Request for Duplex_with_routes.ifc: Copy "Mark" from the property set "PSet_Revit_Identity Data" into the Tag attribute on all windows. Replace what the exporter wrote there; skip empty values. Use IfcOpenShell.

First a look at what the model holds.

```python
import ifcopenshell
import ifcopenshell.util.element

model = ifcopenshell.open("Duplex_with_routes.ifc")
print(model.schema)
windows = model.by_type("IfcWindow")
print(len(windows), "windows")
for e in windows[:8]:
    source = ifcopenshell.util.element.get_pset(e, "PSet_Revit_Identity Data", "Mark")
    target = e.Tag
    print(e.id(), repr(source), repr(target), sep=" | ")
```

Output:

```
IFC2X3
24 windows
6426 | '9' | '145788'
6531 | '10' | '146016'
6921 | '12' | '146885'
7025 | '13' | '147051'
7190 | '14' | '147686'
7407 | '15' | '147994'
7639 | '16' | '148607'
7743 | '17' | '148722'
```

```python
import ifcopenshell
import ifcopenshell.util.element

model = ifcopenshell.open("Duplex_with_routes.ifc")

count = 0
for e in model.by_type("IfcWindow"):
    value = ifcopenshell.util.element.get_pset(e, "PSet_Revit_Identity Data", "Mark")
    current = e.Tag
    if not value or not value.strip() or current == value:
        continue
    e.Tag = value
    count += 1

print(count, "windows updated")

model.write("Duplex_with_routes-out.ifc")
```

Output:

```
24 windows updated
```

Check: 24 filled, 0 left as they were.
